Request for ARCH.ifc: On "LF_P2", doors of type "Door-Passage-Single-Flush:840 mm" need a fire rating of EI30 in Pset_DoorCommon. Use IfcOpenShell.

First a look at what the model holds.

```python
import ifcopenshell
import ifcopenshell.util.element

model = ifcopenshell.open("ARCH.ifc")
print(model.schema)
storey = next(s for s in model.by_type("IfcBuildingStorey") if s.Name == "LF_P2")
doors = [e for e in ifcopenshell.util.element.get_decomposition(storey) if e.is_a("IfcDoor")]
seen = {}
for e in doors:
    element_type = ifcopenshell.util.element.get_type(e)
    key = (element_type.Name if element_type != e and element_type else None, ifcopenshell.util.element.get_pset(e, "Pset_DoorCommon", "FireRating"))
    seen[key] = seen.get(key, 0) + 1
for (name, value), count in sorted(seen.items(), key=str):
    print(count, "x", name, "|", value)
```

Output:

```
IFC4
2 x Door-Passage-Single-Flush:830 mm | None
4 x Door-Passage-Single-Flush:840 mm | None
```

```python
import ifcopenshell
import ifcopenshell.api.pset
import ifcopenshell.util.element

model = ifcopenshell.open("ARCH.ifc")

storey = next(s for s in model.by_type("IfcBuildingStorey") if s.Name == "LF_P2")
doors = [e for e in ifcopenshell.util.element.get_decomposition(storey) if e.is_a("IfcDoor")]

count = 0
for e in doors:
    element_type = ifcopenshell.util.element.get_type(e)
    if element_type in (None, e) or element_type.Name != "Door-Passage-Single-Flush:840 mm":
        continue
    # add_pset returns the element's existing set when there is one.
    pset = ifcopenshell.api.pset.add_pset(model, product=e, name="Pset_DoorCommon")
    ifcopenshell.api.pset.edit_pset(model, pset=pset, properties={"FireRating": "EI30"})
    count += 1

print(count, "doors updated")

model.write("ARCH-out.ifc")
```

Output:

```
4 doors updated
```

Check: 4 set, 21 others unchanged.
